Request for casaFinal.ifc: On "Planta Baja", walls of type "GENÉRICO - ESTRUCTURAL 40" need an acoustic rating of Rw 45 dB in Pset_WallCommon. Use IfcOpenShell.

First a look at what the model holds.

```python
import ifcopenshell
import ifcopenshell.util.element

model = ifcopenshell.open("casaFinal.ifc")
print(model.schema)
storey = next(s for s in model.by_type("IfcBuildingStorey") if s.Name == "Planta Baja")
walls = [e for e in ifcopenshell.util.element.get_decomposition(storey) if e.is_a("IfcWall")]
seen = {}
for e in walls:
    element_type = ifcopenshell.util.element.get_type(e)
    key = (element_type.Name if element_type != e and element_type else None, ifcopenshell.util.element.get_pset(e, "Pset_WallCommon", "AcousticRating"))
    seen[key] = seen.get(key, 0) + 1
for (name, value), count in sorted(seen.items(), key=str):
    print(count, "x", name, "|", value)
```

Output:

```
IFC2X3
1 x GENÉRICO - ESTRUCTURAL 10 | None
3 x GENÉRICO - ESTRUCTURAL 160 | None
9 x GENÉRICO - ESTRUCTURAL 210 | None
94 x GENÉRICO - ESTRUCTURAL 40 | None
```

```python
import ifcopenshell
import ifcopenshell.api.pset
import ifcopenshell.util.element

model = ifcopenshell.open("casaFinal.ifc")

storey = next(s for s in model.by_type("IfcBuildingStorey") if s.Name == "Planta Baja")
walls = [e for e in ifcopenshell.util.element.get_decomposition(storey) if e.is_a("IfcWall")]

count = 0
for e in walls:
    element_type = ifcopenshell.util.element.get_type(e)
    if element_type in (None, e) or element_type.Name != "GENÉRICO - ESTRUCTURAL 40":
        continue
    # add_pset returns the element's existing set when there is one.
    pset = ifcopenshell.api.pset.add_pset(model, product=e, name="Pset_WallCommon")
    ifcopenshell.api.pset.edit_pset(model, pset=pset, properties={"AcousticRating": "Rw 45 dB"})
    count += 1

print(count, "walls updated")

model.write("casaFinal_v2.ifc")
```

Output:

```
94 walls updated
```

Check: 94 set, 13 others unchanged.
